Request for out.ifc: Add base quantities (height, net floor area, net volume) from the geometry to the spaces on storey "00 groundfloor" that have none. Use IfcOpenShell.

First a look at what the model holds.

```python
import ifcopenshell
import ifcopenshell.util.element
import ifcopenshell.util.unit

model = ifcopenshell.open("out.ifc")
print(model.schema)
for unit_type in ("LENGTHUNIT", "AREAUNIT", "VOLUMEUNIT"):
    print(unit_type, ifcopenshell.util.unit.calculate_unit_scale(model, unit_type))
storey = next(s for s in model.by_type("IfcBuildingStorey") if s.Name == "00 groundfloor")
spaces = [e for e in ifcopenshell.util.element.get_decomposition(storey) if e.is_a("IfcSpace")]
for e in sorted(spaces, key=lambda e: e.id()):
    print(e.id(), e.is_a(), e.Name, list(ifcopenshell.util.element.get_psets(e, qtos_only=True)), sep=" | ")
```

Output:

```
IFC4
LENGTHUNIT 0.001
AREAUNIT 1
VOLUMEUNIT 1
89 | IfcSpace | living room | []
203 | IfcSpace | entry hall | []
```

```python
import ifcopenshell
import ifcopenshell.api.pset
import ifcopenshell.geom
import ifcopenshell.util.element
import ifcopenshell.util.shape
import ifcopenshell.util.unit

model = ifcopenshell.open("out.ifc")
unit_scale = ifcopenshell.util.unit.calculate_unit_scale(model)
area_scale = ifcopenshell.util.unit.calculate_unit_scale(model, "AREAUNIT")
volume_scale = ifcopenshell.util.unit.calculate_unit_scale(model, "VOLUMEUNIT")
settings = ifcopenshell.geom.settings()

storey = next(s for s in model.by_type("IfcBuildingStorey") if s.Name == "00 groundfloor")
spaces = [e for e in ifcopenshell.util.element.get_decomposition(storey) if e.is_a("IfcSpace")]

for e in sorted(spaces, key=lambda e: e.id()):
    if ifcopenshell.util.element.get_psets(e, qtos_only=True, should_inherit=False):
        continue
    # Geometry comes back in metres, in the element's own axes.
    shape = ifcopenshell.geom.create_shape(settings, e)
    values = {
        "Height": ifcopenshell.util.shape.get_z(shape.geometry) / unit_scale,
        "NetFloorArea": ifcopenshell.util.shape.get_footprint_area(shape.geometry) / area_scale,
        "NetVolume": ifcopenshell.util.shape.get_volume(shape.geometry) / volume_scale,
    }
    qto = ifcopenshell.api.pset.add_qto(model, product=e, name="Qto_SpaceBaseQuantities")
    ifcopenshell.api.pset.edit_qto(model, qto=qto, properties=values)
    print(e.id(), {k: round(v, 3) for k, v in values.items()})

model.write("out_updated.ifc")
```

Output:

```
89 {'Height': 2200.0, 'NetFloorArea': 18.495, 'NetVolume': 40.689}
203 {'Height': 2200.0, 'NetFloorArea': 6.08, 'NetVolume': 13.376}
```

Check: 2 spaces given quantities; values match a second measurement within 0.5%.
